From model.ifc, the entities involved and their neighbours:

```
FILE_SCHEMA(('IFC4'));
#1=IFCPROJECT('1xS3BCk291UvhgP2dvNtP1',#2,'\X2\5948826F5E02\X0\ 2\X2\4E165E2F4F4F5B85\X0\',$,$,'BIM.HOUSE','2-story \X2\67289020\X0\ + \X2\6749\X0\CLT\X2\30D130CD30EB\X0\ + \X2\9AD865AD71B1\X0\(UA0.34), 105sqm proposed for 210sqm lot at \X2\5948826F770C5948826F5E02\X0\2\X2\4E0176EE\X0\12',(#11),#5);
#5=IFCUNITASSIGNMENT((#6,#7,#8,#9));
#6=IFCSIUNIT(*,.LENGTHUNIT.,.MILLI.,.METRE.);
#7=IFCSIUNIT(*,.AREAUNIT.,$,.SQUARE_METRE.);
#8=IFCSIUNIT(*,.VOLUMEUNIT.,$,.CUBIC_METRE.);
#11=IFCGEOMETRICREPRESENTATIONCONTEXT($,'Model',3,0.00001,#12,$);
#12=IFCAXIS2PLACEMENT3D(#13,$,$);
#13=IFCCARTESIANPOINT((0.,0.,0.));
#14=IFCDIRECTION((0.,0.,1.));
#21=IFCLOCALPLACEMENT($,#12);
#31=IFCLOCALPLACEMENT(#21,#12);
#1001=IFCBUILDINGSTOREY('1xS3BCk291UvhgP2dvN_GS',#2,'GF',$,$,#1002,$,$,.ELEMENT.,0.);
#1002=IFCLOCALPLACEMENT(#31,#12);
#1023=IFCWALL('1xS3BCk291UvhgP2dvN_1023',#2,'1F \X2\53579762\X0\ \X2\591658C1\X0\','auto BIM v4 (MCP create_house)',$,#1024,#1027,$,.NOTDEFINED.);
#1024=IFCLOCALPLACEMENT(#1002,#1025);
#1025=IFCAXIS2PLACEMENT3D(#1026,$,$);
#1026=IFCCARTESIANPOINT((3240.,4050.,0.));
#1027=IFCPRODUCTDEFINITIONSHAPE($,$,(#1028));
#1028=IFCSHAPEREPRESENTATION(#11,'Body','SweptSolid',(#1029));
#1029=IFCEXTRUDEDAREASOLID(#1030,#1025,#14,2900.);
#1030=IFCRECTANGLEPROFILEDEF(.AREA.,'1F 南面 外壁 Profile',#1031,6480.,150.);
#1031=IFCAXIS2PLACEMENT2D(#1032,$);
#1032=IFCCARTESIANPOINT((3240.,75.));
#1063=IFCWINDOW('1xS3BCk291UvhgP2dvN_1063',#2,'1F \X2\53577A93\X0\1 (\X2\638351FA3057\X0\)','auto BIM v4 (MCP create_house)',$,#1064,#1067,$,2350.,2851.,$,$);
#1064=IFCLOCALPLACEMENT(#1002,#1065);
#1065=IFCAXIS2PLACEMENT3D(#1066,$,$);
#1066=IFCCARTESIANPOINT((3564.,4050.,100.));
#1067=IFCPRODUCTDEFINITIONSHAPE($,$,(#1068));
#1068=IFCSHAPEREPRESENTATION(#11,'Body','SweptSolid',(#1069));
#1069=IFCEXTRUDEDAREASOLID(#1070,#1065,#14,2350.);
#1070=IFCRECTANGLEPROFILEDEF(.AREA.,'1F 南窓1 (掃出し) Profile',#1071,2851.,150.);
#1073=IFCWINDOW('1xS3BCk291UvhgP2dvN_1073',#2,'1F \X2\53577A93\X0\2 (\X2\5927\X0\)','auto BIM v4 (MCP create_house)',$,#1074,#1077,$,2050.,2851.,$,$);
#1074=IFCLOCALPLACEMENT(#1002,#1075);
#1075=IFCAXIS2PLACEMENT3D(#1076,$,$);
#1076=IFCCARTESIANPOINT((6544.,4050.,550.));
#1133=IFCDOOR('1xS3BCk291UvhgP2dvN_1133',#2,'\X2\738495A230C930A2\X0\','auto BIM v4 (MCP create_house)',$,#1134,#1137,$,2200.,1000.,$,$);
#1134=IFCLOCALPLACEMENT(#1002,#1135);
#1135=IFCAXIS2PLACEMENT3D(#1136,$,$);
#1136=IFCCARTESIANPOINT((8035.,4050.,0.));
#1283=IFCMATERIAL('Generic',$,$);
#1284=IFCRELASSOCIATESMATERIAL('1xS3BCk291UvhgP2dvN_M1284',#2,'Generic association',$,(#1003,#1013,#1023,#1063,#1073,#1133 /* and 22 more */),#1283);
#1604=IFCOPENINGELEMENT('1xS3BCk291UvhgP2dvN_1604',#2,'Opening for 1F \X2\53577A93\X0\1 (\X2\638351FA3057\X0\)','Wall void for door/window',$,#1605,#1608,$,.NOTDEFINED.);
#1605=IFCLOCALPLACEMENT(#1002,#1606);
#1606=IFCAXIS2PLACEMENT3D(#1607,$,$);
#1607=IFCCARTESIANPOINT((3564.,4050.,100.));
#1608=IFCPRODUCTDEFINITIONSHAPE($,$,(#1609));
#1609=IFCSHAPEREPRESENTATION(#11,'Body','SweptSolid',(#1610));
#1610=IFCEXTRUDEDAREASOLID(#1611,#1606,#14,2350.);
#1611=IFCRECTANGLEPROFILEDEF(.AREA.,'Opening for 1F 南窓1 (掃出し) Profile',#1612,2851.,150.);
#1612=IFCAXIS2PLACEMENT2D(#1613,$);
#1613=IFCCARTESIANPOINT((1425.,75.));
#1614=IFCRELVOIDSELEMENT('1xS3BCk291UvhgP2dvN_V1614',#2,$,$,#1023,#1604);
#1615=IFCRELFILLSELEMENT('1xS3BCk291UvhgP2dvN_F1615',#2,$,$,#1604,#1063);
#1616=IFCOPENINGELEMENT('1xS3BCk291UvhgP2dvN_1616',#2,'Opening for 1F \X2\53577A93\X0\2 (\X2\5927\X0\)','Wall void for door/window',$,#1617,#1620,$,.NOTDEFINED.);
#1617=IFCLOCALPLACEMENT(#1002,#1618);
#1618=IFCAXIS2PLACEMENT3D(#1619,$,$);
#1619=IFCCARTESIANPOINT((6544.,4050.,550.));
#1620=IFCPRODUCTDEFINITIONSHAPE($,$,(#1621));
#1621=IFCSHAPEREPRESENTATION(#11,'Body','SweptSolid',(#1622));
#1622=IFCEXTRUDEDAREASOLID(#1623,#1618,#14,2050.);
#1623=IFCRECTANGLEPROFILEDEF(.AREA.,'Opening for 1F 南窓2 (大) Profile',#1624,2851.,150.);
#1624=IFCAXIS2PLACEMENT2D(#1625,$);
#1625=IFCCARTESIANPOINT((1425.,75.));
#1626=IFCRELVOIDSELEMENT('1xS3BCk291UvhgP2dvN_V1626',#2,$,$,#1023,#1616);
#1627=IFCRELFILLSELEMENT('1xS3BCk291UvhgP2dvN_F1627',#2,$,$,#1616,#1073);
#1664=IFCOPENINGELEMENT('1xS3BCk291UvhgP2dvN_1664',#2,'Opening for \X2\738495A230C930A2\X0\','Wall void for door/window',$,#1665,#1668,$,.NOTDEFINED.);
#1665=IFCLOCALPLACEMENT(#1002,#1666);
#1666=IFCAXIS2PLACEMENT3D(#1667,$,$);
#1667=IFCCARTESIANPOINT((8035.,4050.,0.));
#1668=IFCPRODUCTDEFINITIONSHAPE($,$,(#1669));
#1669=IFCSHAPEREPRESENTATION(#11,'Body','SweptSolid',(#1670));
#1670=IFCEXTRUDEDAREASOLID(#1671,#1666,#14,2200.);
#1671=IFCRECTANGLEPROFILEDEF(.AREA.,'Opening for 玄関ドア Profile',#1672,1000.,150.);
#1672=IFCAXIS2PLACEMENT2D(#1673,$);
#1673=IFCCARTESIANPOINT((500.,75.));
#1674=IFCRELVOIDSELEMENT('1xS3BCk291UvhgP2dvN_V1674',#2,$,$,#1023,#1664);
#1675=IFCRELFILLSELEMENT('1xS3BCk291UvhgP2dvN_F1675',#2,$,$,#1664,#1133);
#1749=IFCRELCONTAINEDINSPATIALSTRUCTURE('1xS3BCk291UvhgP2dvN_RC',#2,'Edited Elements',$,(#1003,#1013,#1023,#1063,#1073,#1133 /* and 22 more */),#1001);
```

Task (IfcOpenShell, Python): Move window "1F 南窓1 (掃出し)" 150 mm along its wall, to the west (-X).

```python
import ifcopenshell
import ifcopenshell.api.geometry
import ifcopenshell.util.placement
import ifcopenshell.util.unit

model = ifcopenshell.open("model.ifc")
unit_scale = ifcopenshell.util.unit.calculate_unit_scale(model)

window = model.by_guid("1xS3BCk291UvhgP2dvN_1063")
opening = window.FillsVoids[0].RelatingOpeningElement
wall = opening.VoidsElements[0].RelatingBuildingElement

wall_matrix = ifcopenshell.util.placement.get_local_placement(wall.ObjectPlacement)
shift = wall_matrix[:3, 0] * -0.15 / unit_scale
before = ifcopenshell.util.placement.get_local_placement(window.ObjectPlacement)[:3, 3].copy()

# The window is not placed relative to its opening, so move both.
for product in (opening, window):
    matrix = ifcopenshell.util.placement.get_local_placement(product.ObjectPlacement)
    matrix[:3, 3] += shift
    ifcopenshell.api.geometry.edit_object_placement(model, product=product, matrix=matrix, is_si=False)

after = ifcopenshell.util.placement.get_local_placement(window.ObjectPlacement)[:3, 3]
print("window moved by", (after - before).round(3) + 0.0)

model.write("model_updated.ifc")
```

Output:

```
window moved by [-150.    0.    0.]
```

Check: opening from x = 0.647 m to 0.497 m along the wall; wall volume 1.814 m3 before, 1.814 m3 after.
